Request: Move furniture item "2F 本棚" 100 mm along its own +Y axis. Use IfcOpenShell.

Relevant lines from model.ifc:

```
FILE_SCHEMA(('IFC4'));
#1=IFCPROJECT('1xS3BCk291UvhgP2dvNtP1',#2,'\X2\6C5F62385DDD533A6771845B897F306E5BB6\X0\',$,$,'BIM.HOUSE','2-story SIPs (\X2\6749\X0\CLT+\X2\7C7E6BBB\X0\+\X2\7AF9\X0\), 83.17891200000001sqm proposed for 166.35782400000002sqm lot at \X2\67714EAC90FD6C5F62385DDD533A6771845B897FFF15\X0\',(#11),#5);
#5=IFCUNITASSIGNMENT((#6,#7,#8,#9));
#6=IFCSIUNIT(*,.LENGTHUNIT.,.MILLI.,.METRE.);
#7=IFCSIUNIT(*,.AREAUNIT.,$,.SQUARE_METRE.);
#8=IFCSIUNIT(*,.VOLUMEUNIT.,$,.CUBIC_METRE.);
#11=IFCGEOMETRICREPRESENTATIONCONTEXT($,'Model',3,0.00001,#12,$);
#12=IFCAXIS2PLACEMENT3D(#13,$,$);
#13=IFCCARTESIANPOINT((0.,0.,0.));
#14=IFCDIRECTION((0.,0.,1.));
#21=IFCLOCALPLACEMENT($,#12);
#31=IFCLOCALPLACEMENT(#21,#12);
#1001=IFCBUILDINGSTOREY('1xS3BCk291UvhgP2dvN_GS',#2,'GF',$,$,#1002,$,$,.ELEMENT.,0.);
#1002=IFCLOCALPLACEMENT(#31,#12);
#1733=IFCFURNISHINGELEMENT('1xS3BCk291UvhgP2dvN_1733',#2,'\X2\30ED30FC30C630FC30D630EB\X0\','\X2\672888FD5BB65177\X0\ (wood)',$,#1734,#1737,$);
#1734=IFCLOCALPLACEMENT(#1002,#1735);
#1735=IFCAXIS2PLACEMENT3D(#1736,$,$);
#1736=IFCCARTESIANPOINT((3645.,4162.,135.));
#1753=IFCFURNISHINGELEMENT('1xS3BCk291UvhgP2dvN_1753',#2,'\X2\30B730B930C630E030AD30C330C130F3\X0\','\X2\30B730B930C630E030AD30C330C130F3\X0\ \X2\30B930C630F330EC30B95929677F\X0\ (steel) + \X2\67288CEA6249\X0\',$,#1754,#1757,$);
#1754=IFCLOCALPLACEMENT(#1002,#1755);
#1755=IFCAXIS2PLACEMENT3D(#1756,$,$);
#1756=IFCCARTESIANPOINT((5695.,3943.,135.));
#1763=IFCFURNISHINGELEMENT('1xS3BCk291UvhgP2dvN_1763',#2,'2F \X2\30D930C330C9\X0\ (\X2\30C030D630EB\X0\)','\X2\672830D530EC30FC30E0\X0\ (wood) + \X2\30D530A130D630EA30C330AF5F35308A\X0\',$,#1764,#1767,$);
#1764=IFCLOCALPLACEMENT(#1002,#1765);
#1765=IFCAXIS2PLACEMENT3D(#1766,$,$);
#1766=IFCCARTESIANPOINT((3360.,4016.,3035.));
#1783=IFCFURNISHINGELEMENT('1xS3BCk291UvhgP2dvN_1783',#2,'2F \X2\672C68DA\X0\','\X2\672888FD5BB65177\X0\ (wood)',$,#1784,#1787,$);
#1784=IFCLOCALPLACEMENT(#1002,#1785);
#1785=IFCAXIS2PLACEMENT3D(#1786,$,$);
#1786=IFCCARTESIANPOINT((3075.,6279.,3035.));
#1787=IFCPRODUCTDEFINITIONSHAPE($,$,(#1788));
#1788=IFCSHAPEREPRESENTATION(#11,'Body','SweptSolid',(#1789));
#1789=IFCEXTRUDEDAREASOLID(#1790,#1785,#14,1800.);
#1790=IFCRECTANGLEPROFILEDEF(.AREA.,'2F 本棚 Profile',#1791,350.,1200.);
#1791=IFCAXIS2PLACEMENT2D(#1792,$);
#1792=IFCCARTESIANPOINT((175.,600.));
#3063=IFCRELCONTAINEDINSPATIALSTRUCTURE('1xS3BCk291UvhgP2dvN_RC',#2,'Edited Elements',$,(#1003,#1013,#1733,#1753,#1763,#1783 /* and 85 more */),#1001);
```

```python
import ifcopenshell
import ifcopenshell.api.geometry
import ifcopenshell.util.placement

model = ifcopenshell.open("model.ifc")

item = model.by_guid("1xS3BCk291UvhgP2dvN_1783")
matrix = ifcopenshell.util.placement.get_local_placement(item.ObjectPlacement)
matrix[:3, 3] += matrix[:3, 1] * 100.0
ifcopenshell.api.geometry.edit_object_placement(model, product=item, matrix=matrix, is_si=False)

print(ifcopenshell.util.placement.get_local_placement(item.ObjectPlacement).round(3) + 0.0)

model.write("model_rev.ifc")
```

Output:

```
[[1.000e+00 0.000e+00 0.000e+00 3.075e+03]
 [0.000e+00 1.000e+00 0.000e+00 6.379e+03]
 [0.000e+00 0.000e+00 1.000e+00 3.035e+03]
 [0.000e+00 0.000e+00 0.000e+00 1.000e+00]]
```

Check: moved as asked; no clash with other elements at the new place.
